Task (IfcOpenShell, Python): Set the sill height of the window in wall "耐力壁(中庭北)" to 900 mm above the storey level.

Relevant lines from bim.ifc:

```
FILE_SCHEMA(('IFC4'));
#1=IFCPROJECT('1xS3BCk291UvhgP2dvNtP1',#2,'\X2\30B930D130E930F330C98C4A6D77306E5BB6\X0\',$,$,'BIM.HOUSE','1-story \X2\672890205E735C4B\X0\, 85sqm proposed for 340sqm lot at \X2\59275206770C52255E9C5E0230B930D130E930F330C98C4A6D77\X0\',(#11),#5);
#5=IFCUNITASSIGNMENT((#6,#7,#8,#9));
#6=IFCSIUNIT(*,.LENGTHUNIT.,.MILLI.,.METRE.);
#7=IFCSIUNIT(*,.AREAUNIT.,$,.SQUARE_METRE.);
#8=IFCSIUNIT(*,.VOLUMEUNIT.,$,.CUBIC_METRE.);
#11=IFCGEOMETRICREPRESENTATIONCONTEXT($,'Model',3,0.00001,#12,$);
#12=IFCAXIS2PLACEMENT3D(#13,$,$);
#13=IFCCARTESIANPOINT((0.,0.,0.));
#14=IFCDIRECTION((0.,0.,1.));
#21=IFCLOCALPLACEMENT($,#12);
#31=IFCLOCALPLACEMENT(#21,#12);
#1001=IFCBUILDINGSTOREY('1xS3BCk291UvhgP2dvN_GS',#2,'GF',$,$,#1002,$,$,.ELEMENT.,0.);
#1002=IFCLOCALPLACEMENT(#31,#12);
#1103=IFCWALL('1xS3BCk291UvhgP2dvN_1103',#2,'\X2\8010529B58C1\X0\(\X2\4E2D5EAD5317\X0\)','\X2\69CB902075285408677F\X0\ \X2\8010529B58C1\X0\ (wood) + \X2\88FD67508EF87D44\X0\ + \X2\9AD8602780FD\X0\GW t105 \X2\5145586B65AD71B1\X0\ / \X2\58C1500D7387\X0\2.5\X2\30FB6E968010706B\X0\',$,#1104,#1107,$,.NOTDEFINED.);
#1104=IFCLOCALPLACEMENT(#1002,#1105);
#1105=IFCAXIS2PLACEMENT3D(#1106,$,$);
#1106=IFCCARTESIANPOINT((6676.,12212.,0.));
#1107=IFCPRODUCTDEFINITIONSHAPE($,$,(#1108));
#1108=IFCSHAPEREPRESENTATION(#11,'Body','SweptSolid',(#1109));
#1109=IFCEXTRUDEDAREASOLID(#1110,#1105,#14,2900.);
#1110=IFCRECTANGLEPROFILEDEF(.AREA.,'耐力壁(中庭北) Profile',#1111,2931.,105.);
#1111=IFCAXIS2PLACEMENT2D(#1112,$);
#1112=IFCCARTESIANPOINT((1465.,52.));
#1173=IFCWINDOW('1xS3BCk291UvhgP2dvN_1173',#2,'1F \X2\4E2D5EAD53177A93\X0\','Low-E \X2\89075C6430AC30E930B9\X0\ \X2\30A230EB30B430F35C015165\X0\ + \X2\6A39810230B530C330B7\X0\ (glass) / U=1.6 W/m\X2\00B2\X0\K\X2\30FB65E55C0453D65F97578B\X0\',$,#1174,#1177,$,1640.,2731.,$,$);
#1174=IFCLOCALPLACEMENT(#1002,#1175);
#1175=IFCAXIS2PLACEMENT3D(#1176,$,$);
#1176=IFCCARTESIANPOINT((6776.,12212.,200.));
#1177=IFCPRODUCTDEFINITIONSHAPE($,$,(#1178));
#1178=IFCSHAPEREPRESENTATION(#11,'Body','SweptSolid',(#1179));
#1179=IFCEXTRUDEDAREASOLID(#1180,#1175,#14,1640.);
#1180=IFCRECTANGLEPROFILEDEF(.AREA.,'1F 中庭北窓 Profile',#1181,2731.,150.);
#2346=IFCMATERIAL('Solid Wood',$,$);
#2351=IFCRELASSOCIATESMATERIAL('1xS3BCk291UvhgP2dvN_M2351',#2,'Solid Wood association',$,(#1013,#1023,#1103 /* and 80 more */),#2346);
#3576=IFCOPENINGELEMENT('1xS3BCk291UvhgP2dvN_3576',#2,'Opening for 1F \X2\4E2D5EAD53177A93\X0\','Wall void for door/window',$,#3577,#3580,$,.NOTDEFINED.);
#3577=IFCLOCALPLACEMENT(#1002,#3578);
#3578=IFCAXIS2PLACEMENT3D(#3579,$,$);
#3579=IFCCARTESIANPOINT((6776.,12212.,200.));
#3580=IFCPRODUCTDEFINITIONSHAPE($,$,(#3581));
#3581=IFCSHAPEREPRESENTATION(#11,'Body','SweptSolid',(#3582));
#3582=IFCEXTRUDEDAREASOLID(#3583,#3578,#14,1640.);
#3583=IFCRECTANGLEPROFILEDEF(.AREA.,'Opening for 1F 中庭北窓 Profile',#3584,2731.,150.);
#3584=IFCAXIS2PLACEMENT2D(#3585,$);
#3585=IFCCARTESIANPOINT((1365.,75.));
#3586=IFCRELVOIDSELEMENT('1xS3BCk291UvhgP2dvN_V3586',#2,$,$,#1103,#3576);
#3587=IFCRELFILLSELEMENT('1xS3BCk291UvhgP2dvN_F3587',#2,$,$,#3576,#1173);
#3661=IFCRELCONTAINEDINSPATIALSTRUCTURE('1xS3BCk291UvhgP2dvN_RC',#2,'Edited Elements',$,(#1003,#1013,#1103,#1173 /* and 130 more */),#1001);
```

```python
import numpy as np
import ifcopenshell
import ifcopenshell.api.geometry
import ifcopenshell.geom
import ifcopenshell.util.element
import ifcopenshell.util.placement
import ifcopenshell.util.shape
import ifcopenshell.util.unit

model = ifcopenshell.open("bim.ifc")
unit_scale = ifcopenshell.util.unit.calculate_unit_scale(model)

window = model.by_guid("1xS3BCk291UvhgP2dvN_1173")
opening = window.FillsVoids[0].RelatingOpeningElement
storey = ifcopenshell.util.element.get_container(window, ifc_class="IfcBuildingStorey")
level = ifcopenshell.util.placement.get_local_placement(storey.ObjectPlacement)[2, 3]

# The opening's origin need not be at the sill, so measure its lowest point.
shape = ifcopenshell.geom.create_shape(ifcopenshell.geom.settings(), opening)
bottom = ifcopenshell.util.shape.get_shape_bottom_elevation(shape, shape.geometry) / unit_scale
dz = level + 900.0 - bottom

shift = np.array([0.0, 0.0, dz])
# The window is not placed relative to its opening, so move both.
for product in (opening, window):
    matrix = ifcopenshell.util.placement.get_local_placement(product.ObjectPlacement)
    matrix[:3, 3] += shift
    ifcopenshell.api.geometry.edit_object_placement(model, product=product, matrix=matrix, is_si=False)

print(f"moved by {dz * unit_scale:+.3f} m")

model.write("bim_rev.ifc")
```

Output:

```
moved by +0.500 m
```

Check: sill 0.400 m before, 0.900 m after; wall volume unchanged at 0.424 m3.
